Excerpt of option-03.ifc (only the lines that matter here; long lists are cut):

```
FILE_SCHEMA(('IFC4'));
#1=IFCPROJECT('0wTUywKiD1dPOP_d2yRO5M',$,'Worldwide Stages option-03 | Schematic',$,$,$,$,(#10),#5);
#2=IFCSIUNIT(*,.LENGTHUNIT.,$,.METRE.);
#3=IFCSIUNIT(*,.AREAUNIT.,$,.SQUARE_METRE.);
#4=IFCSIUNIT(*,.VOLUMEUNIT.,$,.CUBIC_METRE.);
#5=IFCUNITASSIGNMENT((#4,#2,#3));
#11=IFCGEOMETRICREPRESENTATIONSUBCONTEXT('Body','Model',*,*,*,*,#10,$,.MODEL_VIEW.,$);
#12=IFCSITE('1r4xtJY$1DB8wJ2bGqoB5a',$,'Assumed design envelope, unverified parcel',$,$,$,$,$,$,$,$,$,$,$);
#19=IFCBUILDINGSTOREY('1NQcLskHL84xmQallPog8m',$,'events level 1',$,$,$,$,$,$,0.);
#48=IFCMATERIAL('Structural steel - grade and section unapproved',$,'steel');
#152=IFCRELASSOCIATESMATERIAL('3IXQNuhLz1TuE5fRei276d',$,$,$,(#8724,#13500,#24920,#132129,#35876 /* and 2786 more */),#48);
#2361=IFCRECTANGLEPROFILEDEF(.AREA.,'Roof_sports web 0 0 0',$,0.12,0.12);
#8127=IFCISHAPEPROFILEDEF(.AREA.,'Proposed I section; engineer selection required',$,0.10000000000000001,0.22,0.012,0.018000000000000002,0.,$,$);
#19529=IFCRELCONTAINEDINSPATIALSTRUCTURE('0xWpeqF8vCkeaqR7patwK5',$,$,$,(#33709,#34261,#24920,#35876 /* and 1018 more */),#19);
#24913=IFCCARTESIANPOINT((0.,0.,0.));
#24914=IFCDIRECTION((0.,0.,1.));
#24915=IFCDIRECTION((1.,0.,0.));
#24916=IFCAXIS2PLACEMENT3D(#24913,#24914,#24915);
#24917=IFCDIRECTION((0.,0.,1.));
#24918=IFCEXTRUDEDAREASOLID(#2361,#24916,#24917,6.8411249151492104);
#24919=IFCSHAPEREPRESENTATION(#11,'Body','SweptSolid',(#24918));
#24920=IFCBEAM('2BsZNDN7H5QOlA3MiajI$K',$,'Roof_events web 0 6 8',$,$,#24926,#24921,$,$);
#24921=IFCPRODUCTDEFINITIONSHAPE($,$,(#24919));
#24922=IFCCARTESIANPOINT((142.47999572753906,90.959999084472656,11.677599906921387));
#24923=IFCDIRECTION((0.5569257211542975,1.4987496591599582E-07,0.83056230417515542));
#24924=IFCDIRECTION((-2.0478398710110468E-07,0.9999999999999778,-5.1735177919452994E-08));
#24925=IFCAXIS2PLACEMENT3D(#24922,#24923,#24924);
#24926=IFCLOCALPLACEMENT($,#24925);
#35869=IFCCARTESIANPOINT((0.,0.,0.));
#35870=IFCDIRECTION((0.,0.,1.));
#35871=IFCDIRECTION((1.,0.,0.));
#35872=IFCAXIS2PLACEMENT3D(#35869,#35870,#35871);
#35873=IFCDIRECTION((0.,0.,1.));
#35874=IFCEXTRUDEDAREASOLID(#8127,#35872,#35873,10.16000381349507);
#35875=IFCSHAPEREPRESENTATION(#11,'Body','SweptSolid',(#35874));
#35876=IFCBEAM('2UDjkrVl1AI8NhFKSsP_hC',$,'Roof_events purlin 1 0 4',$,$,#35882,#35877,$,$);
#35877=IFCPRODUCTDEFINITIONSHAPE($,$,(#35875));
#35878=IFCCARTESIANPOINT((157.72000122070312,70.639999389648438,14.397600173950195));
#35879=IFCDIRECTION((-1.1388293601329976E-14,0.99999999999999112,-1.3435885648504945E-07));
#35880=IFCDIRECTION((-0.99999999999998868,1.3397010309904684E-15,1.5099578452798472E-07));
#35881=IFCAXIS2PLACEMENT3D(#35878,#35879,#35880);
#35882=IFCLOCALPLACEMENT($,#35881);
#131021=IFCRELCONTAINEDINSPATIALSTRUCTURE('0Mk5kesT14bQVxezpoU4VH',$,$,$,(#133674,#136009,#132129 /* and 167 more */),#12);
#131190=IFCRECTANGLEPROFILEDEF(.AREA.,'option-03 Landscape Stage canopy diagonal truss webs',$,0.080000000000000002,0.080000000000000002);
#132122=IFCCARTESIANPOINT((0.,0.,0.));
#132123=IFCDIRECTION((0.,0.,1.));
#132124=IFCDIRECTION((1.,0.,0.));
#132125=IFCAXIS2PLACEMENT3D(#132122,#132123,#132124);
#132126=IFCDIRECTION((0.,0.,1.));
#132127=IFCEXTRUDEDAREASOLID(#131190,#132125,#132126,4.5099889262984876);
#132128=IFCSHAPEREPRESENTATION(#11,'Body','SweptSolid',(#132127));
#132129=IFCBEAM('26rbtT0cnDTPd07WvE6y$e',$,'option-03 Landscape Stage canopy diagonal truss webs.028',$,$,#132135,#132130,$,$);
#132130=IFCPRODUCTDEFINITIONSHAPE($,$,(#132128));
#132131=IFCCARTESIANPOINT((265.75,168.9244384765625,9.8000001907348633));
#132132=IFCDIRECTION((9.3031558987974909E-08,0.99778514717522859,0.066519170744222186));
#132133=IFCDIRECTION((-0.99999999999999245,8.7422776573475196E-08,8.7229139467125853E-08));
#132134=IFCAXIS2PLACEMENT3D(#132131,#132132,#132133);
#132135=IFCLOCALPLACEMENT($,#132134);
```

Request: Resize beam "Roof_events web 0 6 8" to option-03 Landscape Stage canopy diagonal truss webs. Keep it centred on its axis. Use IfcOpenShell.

```python
import ifcopenshell
import ifcopenshell.util.element
import ifcopenshell.util.representation

model = ifcopenshell.open("option-03.ifc")

member = model.by_guid("2BsZNDN7H5QOlA3MiajI$K")
source = next(p for p in model.by_type("IfcRectangleProfileDef") if p.ProfileName == "option-03 Landscape Stage canopy diagonal truss webs")

body = ifcopenshell.util.representation.get_representation(member, "Model", "Body")
solid = body.Items[0]
old_profile = solid.SweptArea

# Copy the section's sizes but keep this member's own profile position.
profile = ifcopenshell.util.element.copy(model, source)
profile.Position = old_profile.Position
solid.SweptArea = profile
if not model.get_total_inverses(old_profile):
    ifcopenshell.util.element.remove_deep2(model, old_profile)

print(solid.SweptArea)

model.write("option-03_updated.ifc")
```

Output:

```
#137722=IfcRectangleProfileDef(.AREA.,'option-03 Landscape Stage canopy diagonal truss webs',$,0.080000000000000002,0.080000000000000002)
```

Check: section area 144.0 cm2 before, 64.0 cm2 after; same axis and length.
